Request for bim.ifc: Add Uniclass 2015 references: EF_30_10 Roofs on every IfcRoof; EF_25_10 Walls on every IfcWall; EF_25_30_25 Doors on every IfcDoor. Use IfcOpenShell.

First a look at what the model holds.

```python
import ifcopenshell

model = ifcopenshell.open("bim.ifc")
print(model.schema)
print("classifications:", [c.Name for c in model.by_type("IfcClassification")])
for ifc_class in ("IfcDoor", "IfcRoof", "IfcStair", "IfcWall", "IfcWindow"):
    print(ifc_class, len(model.by_type(ifc_class)))
```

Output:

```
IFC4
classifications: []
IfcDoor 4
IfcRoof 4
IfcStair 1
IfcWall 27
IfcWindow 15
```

```python
import ifcopenshell
import ifcopenshell.api.classification

model = ifcopenshell.open("bim.ifc")

system = ifcopenshell.api.classification.add_classification(model, classification="Uniclass 2015")

codes = {
    "IfcRoof": ("EF_30_10", "Roofs"),
    "IfcWall": ("EF_25_10", "Walls"),
    "IfcDoor": ("EF_25_30_25", "Doors"),
}
for ifc_class, (code, name) in codes.items():
    products = model.by_type(ifc_class)
    ifcopenshell.api.classification.add_reference(
        model, products=products, classification=system, identification=code, name=name
    )
    print(code, len(products))

model.write("bim_edited.ifc")
```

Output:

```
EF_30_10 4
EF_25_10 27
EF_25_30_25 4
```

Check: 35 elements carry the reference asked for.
